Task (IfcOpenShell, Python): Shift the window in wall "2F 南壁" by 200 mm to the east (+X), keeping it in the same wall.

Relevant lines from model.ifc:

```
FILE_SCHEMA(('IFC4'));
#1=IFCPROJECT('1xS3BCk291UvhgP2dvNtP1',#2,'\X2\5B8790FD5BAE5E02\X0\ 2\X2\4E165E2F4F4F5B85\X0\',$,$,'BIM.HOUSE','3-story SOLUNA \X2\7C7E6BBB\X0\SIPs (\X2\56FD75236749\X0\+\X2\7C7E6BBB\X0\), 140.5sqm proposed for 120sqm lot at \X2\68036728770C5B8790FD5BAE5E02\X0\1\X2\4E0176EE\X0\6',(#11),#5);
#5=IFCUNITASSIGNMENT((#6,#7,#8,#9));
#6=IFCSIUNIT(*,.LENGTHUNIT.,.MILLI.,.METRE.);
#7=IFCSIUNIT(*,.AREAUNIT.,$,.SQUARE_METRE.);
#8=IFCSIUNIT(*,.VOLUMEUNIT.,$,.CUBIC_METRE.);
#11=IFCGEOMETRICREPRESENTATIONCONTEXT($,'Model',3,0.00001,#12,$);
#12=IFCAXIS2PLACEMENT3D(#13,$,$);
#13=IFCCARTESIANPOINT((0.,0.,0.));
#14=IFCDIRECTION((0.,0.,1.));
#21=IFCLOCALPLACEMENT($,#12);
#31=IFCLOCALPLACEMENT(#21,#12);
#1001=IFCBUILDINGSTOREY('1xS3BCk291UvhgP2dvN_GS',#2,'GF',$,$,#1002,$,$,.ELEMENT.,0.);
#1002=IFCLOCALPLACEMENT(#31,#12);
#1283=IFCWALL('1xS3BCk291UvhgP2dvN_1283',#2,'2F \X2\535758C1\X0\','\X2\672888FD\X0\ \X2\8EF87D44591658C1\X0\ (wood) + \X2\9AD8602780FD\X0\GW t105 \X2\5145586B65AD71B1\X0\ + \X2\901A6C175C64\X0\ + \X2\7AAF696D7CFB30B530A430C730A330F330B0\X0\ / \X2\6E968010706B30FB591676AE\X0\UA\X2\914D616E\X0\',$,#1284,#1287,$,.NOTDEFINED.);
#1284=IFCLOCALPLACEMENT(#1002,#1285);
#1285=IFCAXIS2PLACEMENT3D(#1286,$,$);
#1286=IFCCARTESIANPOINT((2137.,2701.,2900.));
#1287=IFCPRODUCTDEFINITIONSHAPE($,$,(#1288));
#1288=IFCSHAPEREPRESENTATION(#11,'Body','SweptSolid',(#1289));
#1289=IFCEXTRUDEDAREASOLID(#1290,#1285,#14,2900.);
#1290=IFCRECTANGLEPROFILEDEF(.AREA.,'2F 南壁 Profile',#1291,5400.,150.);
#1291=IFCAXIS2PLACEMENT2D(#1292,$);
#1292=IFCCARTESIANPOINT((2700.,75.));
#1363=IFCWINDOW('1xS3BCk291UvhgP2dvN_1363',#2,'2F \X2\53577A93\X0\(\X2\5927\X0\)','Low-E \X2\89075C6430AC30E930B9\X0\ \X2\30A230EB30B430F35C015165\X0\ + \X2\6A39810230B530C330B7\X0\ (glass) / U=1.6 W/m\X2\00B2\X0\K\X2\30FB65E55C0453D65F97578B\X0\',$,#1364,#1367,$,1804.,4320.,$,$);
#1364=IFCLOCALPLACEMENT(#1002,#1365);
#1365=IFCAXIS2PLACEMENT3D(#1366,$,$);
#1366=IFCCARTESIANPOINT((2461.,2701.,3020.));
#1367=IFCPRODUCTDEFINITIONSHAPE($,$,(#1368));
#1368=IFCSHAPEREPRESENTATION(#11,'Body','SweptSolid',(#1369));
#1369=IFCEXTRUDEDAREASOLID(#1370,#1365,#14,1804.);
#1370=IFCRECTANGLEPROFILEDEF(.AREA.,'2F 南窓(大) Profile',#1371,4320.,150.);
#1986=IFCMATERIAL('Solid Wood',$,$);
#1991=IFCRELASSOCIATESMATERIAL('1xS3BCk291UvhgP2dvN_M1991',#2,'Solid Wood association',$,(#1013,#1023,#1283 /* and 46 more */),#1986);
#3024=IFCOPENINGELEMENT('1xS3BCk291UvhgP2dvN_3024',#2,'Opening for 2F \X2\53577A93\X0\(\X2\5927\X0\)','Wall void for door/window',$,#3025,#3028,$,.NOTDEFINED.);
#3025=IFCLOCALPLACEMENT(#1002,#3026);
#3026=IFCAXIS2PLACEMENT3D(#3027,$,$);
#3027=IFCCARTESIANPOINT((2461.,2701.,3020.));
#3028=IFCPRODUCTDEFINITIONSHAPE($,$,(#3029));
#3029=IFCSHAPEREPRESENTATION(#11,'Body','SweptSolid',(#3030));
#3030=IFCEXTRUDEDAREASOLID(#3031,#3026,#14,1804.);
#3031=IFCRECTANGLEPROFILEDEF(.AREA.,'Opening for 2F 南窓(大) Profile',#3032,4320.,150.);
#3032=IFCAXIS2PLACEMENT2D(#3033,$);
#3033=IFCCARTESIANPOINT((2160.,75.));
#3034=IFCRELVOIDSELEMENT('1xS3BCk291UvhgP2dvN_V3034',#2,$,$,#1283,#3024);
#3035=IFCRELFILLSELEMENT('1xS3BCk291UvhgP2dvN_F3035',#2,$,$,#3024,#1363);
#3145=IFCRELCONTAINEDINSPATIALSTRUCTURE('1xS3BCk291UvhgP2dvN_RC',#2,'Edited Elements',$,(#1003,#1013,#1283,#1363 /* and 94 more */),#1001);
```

```python
import ifcopenshell
import ifcopenshell.api.geometry
import ifcopenshell.util.placement

model = ifcopenshell.open("model.ifc")

window = model.by_guid("1xS3BCk291UvhgP2dvN_1363")
opening = window.FillsVoids[0].RelatingOpeningElement
wall = opening.VoidsElements[0].RelatingBuildingElement

wall_matrix = ifcopenshell.util.placement.get_local_placement(wall.ObjectPlacement)
shift = wall_matrix[:3, 0] * 200.0
before = ifcopenshell.util.placement.get_local_placement(window.ObjectPlacement)[:3, 3].copy()

# The window is not placed relative to its opening, so move both.
for product in (opening, window):
    matrix = ifcopenshell.util.placement.get_local_placement(product.ObjectPlacement)
    matrix[:3, 3] += shift
    ifcopenshell.api.geometry.edit_object_placement(model, product=product, matrix=matrix, is_si=False)

after = ifcopenshell.util.placement.get_local_placement(window.ObjectPlacement)[:3, 3]
print("window moved by", (after - before).round(3) + 0.0)

model.write("model_edited.ifc")
```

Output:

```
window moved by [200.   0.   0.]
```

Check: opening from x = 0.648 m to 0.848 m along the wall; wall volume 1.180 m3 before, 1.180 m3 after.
